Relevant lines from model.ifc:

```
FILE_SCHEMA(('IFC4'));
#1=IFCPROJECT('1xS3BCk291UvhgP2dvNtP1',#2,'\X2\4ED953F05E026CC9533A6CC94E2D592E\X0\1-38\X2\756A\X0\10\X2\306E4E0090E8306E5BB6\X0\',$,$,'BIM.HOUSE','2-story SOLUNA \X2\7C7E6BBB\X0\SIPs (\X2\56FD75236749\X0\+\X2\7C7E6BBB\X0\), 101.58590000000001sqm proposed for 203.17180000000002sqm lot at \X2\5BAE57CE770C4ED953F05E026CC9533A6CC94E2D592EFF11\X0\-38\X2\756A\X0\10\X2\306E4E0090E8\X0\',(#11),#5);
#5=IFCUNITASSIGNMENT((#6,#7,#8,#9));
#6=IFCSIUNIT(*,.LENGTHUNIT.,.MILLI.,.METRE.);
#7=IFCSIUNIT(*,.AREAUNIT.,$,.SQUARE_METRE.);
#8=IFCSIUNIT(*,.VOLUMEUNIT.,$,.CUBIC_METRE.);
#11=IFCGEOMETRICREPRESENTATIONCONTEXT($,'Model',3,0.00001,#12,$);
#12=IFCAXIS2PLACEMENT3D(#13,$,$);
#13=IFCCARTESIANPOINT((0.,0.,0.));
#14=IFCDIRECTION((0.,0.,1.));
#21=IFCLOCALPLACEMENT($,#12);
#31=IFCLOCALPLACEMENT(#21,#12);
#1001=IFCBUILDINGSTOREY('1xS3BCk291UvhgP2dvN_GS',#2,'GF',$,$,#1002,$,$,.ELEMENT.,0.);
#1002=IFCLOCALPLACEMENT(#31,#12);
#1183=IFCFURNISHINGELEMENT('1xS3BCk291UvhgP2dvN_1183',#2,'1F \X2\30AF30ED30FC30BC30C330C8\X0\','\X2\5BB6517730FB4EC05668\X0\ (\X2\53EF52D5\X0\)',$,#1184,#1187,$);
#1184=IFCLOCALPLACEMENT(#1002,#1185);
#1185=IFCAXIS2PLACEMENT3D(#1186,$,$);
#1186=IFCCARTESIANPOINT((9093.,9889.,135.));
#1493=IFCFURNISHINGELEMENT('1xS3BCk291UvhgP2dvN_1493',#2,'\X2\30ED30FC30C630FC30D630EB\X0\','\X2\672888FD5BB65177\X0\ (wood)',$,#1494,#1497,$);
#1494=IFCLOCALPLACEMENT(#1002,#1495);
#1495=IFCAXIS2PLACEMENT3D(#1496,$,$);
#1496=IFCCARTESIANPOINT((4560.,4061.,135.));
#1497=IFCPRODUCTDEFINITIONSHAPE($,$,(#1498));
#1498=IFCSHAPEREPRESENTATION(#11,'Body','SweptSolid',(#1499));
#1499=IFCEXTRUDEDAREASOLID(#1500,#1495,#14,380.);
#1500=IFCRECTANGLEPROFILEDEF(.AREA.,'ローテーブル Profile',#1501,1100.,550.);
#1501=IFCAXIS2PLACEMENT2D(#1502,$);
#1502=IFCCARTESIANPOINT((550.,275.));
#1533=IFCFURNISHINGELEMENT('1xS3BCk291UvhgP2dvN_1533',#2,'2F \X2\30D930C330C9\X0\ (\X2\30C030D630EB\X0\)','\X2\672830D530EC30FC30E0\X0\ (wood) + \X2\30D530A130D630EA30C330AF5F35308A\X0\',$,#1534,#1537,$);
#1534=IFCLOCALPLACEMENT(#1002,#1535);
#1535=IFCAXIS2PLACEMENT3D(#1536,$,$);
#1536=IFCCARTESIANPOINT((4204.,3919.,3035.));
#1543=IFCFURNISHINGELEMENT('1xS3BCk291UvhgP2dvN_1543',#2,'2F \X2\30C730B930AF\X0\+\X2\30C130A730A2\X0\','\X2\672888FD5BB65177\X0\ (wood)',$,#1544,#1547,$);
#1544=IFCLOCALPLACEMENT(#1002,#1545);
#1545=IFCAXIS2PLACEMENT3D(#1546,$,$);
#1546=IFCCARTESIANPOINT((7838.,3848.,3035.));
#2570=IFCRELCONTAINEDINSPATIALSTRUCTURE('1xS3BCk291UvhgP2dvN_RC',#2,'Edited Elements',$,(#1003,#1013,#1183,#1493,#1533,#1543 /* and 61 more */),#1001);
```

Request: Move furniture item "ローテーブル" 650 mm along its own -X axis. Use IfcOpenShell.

```python
import ifcopenshell
import ifcopenshell.api.geometry
import ifcopenshell.util.placement

model = ifcopenshell.open("model.ifc")

item = model.by_id(1493)
matrix = ifcopenshell.util.placement.get_local_placement(item.ObjectPlacement)
matrix[:3, 3] -= matrix[:3, 0] * 650.0
ifcopenshell.api.geometry.edit_object_placement(model, product=item, matrix=matrix, is_si=False)

print(ifcopenshell.util.placement.get_local_placement(item.ObjectPlacement).round(3) + 0.0)

model.write("model-out.ifc")
```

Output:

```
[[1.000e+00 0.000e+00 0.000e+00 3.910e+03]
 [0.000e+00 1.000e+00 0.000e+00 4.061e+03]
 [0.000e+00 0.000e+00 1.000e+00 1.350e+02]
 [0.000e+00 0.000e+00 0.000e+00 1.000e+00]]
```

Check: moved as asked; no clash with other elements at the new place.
